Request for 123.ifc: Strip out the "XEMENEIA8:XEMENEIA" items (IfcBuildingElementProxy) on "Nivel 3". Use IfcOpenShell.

First a look at what the model holds.

```python
import ifcopenshell
import ifcopenshell.util.element

model = ifcopenshell.open("123.ifc")
print(model.schema)
storey = next(s for s in model.by_type("IfcBuildingStorey") if s.Name == "Nivel 3")
proxies = [e for e in ifcopenshell.util.element.get_decomposition(storey) if e.is_a("IfcBuildingElementProxy")]
seen = {}
for e in proxies:
    element_type = ifcopenshell.util.element.get_type(e)
    name = element_type.Name if element_type not in (None, e) else None
    seen[name] = seen.get(name, 0) + 1
for name, count in sorted(seen.items(), key=str):
    print(count, "x", name)
```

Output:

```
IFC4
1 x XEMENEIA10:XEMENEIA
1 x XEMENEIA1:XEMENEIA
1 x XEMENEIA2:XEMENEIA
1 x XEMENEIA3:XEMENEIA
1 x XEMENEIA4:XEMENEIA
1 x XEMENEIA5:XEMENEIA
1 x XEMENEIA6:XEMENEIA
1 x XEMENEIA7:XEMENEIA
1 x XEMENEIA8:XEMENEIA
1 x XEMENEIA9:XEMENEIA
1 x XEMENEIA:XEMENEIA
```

```python
import ifcopenshell
import ifcopenshell.api.root
import ifcopenshell.util.element

model = ifcopenshell.open("123.ifc")

storey = next(s for s in model.by_type("IfcBuildingStorey") if s.Name == "Nivel 3")
proxies = [e for e in ifcopenshell.util.element.get_decomposition(storey) if e.is_a("IfcBuildingElementProxy")]
targets = [e for e in proxies if (t := ifcopenshell.util.element.get_type(e)) not in (None, e) and t.Name == "XEMENEIA8:XEMENEIA"]

for e in targets:
    ifcopenshell.api.root.remove_product(model, product=e)
print(len(targets), "removed")

model.write("123-out.ifc")
```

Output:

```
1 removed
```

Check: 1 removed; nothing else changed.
